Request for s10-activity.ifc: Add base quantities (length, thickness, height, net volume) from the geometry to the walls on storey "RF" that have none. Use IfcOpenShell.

First a look at what the model holds.

```python
import ifcopenshell
import ifcopenshell.util.element
import ifcopenshell.util.unit

model = ifcopenshell.open("s10-activity.ifc")
print(model.schema)
for unit_type in ("LENGTHUNIT", "AREAUNIT", "VOLUMEUNIT"):
    print(unit_type, ifcopenshell.util.unit.calculate_unit_scale(model, unit_type))
storey = next(s for s in model.by_type("IfcBuildingStorey") if s.Name == "RF")
walls = [e for e in ifcopenshell.util.element.get_decomposition(storey) if e.is_a("IfcWall")]
for e in sorted(walls, key=lambda e: e.id()):
    print(e.id(), e.is_a(), e.Name, list(ifcopenshell.util.element.get_psets(e, qtos_only=True)), sep=" | ")
```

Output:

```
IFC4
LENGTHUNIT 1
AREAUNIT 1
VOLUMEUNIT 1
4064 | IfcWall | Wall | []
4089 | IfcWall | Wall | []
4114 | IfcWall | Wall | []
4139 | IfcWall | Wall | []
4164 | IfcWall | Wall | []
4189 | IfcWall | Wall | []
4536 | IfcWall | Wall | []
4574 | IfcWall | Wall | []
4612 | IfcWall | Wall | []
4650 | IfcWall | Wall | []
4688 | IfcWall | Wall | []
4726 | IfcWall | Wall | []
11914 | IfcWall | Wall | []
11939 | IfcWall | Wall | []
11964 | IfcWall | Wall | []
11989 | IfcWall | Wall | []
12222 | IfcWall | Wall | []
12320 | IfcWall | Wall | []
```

```python
import ifcopenshell
import ifcopenshell.api.pset
import ifcopenshell.geom
import ifcopenshell.util.element
import ifcopenshell.util.shape
import ifcopenshell.util.unit

model = ifcopenshell.open("s10-activity.ifc")
unit_scale = ifcopenshell.util.unit.calculate_unit_scale(model)
volume_scale = ifcopenshell.util.unit.calculate_unit_scale(model, "VOLUMEUNIT")
settings = ifcopenshell.geom.settings()

storey = next(s for s in model.by_type("IfcBuildingStorey") if s.Name == "RF")
walls = [e for e in ifcopenshell.util.element.get_decomposition(storey) if e.is_a("IfcWall")]

for e in sorted(walls, key=lambda e: e.id()):
    if ifcopenshell.util.element.get_psets(e, qtos_only=True, should_inherit=False):
        continue
    # Geometry comes back in metres, in the element's own axes.
    shape = ifcopenshell.geom.create_shape(settings, e)
    values = {
        "Length": ifcopenshell.util.shape.get_x(shape.geometry) / unit_scale,
        "Width": ifcopenshell.util.shape.get_y(shape.geometry) / unit_scale,
        "Height": ifcopenshell.util.shape.get_z(shape.geometry) / unit_scale,
        "NetVolume": ifcopenshell.util.shape.get_volume(shape.geometry) / volume_scale,
    }
    qto = ifcopenshell.api.pset.add_qto(model, product=e, name="Qto_WallBaseQuantities")
    ifcopenshell.api.pset.edit_qto(model, qto=qto, properties=values)
    print(e.id(), {k: round(v, 3) for k, v in values.items()})

model.write("s10-activity_updated.ifc")
```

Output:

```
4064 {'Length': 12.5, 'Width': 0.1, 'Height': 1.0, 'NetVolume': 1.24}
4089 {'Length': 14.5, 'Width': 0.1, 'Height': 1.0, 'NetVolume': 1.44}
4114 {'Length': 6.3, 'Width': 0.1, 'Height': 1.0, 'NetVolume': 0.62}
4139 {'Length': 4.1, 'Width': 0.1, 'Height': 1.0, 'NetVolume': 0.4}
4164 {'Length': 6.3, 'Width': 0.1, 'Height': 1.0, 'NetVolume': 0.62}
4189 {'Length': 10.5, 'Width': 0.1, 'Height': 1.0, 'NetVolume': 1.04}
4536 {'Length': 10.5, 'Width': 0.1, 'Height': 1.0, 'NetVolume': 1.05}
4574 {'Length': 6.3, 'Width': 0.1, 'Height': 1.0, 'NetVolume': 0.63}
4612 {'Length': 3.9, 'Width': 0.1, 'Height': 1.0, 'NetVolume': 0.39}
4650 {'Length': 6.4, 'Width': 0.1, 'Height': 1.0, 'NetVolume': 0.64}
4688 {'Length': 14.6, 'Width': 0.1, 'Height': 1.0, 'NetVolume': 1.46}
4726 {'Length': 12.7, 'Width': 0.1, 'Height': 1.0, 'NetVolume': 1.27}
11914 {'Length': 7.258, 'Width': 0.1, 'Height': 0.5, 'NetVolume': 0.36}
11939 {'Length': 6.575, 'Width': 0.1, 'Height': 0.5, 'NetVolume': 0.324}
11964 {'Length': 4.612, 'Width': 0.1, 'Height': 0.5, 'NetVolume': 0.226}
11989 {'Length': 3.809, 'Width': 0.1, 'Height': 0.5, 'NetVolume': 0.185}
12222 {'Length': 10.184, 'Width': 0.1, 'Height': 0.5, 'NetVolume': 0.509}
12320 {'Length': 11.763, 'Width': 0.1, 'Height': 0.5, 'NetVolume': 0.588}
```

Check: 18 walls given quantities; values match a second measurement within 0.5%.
